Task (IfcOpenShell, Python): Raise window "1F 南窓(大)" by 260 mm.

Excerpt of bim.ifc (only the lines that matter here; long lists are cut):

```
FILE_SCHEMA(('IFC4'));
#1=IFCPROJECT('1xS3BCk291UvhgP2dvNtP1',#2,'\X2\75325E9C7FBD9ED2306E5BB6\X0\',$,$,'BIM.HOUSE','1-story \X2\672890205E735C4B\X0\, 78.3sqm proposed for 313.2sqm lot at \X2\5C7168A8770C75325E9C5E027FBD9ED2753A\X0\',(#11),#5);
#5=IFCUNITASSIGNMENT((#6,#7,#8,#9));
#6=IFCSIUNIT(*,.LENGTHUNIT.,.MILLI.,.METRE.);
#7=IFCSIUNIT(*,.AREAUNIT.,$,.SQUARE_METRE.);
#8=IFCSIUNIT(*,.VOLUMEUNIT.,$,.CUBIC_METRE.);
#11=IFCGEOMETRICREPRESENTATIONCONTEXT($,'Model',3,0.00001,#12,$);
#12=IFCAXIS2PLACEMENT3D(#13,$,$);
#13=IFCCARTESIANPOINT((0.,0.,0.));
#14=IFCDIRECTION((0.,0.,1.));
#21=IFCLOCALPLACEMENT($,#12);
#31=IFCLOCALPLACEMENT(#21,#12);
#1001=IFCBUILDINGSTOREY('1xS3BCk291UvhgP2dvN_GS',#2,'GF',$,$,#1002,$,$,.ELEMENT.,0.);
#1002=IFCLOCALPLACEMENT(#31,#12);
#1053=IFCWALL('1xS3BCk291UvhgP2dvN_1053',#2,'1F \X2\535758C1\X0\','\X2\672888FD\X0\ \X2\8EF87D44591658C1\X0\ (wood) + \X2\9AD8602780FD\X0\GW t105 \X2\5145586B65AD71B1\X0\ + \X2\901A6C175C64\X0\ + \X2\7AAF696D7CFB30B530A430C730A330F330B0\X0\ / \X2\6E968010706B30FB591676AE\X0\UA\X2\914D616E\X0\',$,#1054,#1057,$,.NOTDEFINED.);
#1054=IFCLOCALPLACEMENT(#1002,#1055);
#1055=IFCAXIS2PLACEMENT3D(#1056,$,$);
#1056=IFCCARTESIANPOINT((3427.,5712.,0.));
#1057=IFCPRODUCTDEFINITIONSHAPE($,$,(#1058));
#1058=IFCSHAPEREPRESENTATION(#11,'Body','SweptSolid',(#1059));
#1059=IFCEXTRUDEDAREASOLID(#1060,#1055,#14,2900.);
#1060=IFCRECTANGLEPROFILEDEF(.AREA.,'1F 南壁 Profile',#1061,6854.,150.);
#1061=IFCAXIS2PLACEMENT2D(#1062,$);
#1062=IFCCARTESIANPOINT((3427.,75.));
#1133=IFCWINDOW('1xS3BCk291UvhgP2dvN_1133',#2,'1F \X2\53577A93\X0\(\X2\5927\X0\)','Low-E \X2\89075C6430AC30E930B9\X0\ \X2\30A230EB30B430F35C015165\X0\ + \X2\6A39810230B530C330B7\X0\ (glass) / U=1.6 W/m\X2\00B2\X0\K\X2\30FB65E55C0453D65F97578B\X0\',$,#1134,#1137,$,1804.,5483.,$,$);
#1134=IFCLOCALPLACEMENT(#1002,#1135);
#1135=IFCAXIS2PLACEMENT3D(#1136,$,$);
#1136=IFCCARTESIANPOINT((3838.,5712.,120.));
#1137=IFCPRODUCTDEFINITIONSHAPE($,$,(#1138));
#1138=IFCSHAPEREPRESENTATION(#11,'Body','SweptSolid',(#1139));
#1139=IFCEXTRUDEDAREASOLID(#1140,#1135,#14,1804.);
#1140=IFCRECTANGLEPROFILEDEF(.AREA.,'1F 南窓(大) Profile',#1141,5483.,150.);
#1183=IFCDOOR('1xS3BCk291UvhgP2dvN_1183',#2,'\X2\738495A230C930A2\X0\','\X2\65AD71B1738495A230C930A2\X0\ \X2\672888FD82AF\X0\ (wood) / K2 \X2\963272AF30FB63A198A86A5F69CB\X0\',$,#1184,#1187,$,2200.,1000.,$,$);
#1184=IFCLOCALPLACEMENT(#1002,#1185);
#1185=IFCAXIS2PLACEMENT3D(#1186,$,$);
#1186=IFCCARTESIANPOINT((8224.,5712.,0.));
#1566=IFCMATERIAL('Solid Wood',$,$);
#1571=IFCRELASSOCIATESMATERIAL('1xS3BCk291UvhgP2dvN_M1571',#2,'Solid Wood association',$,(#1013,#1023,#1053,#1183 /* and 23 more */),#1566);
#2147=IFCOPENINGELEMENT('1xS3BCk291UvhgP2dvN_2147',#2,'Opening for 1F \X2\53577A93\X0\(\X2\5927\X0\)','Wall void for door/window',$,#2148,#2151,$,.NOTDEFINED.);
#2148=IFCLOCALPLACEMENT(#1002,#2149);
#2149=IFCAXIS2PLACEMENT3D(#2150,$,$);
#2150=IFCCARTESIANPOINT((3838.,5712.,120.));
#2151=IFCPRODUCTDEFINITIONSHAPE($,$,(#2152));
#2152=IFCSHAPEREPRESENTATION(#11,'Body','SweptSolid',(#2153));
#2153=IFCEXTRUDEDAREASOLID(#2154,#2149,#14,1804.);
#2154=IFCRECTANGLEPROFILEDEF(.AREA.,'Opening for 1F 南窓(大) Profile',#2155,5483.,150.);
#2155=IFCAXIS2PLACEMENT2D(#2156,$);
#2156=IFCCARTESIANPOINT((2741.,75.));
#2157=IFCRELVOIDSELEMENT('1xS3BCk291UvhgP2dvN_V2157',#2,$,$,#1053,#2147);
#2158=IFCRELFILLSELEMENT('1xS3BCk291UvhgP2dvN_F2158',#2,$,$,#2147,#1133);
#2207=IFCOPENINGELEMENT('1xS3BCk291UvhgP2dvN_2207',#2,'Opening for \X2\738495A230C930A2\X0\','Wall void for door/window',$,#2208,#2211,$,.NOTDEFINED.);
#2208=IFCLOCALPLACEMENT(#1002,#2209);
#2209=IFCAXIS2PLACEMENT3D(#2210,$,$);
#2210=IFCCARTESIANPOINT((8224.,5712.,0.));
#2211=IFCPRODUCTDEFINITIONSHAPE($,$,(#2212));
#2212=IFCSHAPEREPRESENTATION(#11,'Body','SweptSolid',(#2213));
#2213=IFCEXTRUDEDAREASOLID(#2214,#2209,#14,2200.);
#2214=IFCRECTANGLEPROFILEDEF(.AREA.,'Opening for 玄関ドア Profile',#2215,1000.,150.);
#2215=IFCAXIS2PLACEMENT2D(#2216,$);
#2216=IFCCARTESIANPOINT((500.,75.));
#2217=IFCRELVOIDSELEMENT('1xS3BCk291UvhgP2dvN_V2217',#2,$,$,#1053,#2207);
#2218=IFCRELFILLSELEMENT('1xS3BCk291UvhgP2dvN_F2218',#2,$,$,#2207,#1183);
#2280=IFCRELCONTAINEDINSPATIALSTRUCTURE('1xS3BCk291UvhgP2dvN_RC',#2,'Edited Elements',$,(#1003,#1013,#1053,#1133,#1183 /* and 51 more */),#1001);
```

```python
import numpy as np
import ifcopenshell
import ifcopenshell.api.geometry
import ifcopenshell.util.placement
import ifcopenshell.util.unit

model = ifcopenshell.open("bim.ifc")
unit_scale = ifcopenshell.util.unit.calculate_unit_scale(model)

window = model.by_id(1133)
opening = window.FillsVoids[0].RelatingOpeningElement
dz = 260.0

shift = np.array([0.0, 0.0, dz])
# The window is not placed relative to its opening, so move both.
for product in (opening, window):
    matrix = ifcopenshell.util.placement.get_local_placement(product.ObjectPlacement)
    matrix[:3, 3] += shift
    ifcopenshell.api.geometry.edit_object_placement(model, product=product, matrix=matrix, is_si=False)

print(f"moved by {dz * unit_scale:+.3f} m")

model.write("bim-out.ifc")
```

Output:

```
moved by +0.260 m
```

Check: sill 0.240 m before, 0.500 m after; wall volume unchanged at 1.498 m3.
